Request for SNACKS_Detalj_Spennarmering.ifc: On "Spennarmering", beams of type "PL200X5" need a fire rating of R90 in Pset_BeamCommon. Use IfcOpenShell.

First a look at what the model holds.

```python
import ifcopenshell
import ifcopenshell.util.element

model = ifcopenshell.open("SNACKS_Detalj_Spennarmering.ifc")
print(model.schema)
storey = next(s for s in model.by_type("IfcBuildingStorey") if s.Name == "Spennarmering")
beams = [e for e in ifcopenshell.util.element.get_decomposition(storey) if e.is_a("IfcBeam")]
seen = {}
for e in beams:
    element_type = ifcopenshell.util.element.get_type(e)
    key = (element_type.Name if element_type != e and element_type else None, ifcopenshell.util.element.get_pset(e, "Pset_BeamCommon", "FireRating"))
    seen[key] = seen.get(key, 0) + 1
for (name, value), count in sorted(seen.items(), key=str):
    print(count, "x", name, "|", value)
```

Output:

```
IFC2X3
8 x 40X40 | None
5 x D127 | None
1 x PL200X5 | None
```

```python
import ifcopenshell
import ifcopenshell.api.pset
import ifcopenshell.util.element

model = ifcopenshell.open("SNACKS_Detalj_Spennarmering.ifc")

storey = next(s for s in model.by_type("IfcBuildingStorey") if s.Name == "Spennarmering")
beams = [e for e in ifcopenshell.util.element.get_decomposition(storey) if e.is_a("IfcBeam")]

count = 0
for e in beams:
    element_type = ifcopenshell.util.element.get_type(e)
    if element_type in (None, e) or element_type.Name != "PL200X5":
        continue
    # add_pset returns the element's existing set when there is one.
    pset = ifcopenshell.api.pset.add_pset(model, product=e, name="Pset_BeamCommon")
    ifcopenshell.api.pset.edit_pset(model, pset=pset, properties={"FireRating": "R90"})
    count += 1

print(count, "beams updated")

model.write("SNACKS_Detalj_Spennarmering_rev.ifc")
```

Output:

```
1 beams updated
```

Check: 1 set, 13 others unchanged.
